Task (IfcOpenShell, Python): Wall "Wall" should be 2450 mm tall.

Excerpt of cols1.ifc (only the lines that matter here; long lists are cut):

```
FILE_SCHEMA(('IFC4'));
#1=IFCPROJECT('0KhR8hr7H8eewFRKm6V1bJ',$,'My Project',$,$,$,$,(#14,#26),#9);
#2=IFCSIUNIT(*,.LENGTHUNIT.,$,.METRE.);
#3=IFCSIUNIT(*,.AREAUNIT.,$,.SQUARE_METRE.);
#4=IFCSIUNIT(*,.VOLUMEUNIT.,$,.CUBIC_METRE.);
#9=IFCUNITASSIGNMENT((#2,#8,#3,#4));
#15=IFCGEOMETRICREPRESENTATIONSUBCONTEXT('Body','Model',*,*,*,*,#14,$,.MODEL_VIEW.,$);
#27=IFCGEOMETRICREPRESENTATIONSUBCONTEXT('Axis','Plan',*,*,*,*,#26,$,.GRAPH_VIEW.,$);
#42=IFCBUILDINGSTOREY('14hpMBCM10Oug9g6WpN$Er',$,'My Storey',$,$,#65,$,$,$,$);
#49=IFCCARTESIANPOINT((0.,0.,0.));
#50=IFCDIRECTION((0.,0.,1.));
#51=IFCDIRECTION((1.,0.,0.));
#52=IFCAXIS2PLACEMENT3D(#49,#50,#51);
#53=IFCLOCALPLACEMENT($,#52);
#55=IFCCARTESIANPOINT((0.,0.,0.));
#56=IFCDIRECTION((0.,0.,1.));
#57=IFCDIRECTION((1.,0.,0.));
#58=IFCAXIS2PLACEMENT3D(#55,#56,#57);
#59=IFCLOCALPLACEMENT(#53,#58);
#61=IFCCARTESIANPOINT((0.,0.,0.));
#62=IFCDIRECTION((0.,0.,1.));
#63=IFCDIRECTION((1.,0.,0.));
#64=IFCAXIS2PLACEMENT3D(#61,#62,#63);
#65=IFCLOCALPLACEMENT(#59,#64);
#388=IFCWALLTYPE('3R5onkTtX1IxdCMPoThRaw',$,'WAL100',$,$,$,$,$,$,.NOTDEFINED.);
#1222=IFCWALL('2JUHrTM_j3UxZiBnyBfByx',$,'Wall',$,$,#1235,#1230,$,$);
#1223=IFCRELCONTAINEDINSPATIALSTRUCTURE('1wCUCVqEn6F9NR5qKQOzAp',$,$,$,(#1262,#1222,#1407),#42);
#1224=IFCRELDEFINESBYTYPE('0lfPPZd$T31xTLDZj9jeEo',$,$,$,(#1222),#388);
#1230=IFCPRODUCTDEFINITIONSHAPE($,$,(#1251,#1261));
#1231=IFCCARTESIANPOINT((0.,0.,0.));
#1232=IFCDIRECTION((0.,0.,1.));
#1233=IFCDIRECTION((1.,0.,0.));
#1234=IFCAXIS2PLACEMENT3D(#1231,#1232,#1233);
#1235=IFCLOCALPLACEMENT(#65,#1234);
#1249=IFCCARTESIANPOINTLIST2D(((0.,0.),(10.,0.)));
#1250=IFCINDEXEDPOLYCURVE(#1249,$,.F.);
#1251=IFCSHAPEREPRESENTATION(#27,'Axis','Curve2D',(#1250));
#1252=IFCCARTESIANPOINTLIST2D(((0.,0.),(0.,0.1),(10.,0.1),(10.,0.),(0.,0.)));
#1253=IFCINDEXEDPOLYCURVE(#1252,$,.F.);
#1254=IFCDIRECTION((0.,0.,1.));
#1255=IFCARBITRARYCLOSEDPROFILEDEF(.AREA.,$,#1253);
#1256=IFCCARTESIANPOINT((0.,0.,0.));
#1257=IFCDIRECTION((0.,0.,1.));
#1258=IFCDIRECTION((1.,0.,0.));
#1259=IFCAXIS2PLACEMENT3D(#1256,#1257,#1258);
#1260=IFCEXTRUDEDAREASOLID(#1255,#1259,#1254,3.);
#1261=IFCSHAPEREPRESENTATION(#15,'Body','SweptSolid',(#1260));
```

```python
import ifcopenshell
import ifcopenshell.geom
import ifcopenshell.util.representation
import ifcopenshell.util.shape
import ifcopenshell.util.unit

model = ifcopenshell.open("cols1.ifc")
unit_scale = ifcopenshell.util.unit.calculate_unit_scale(model)
settings = ifcopenshell.geom.settings()


def volume(element):
    """Net volume in cubic metres, openings subtracted."""
    shape = ifcopenshell.geom.create_shape(settings, element)
    return ifcopenshell.util.shape.get_volume(shape.geometry)


wall = model.by_guid("2JUHrTM_j3UxZiBnyBfByx")
before = volume(wall)

body = ifcopenshell.util.representation.get_representation(wall, "Model", "Body")
solid = body.Items[0]
old_height = solid.Depth
solid.Depth = 2.45 / unit_scale
after = volume(wall)

print(f"height {old_height:g} -> {solid.Depth:g}, volume {before:.3f} -> {after:.3f} m3")

model.write("cols1_v2.ifc")
```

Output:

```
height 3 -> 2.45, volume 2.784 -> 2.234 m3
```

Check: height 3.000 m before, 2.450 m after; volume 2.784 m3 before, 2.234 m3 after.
